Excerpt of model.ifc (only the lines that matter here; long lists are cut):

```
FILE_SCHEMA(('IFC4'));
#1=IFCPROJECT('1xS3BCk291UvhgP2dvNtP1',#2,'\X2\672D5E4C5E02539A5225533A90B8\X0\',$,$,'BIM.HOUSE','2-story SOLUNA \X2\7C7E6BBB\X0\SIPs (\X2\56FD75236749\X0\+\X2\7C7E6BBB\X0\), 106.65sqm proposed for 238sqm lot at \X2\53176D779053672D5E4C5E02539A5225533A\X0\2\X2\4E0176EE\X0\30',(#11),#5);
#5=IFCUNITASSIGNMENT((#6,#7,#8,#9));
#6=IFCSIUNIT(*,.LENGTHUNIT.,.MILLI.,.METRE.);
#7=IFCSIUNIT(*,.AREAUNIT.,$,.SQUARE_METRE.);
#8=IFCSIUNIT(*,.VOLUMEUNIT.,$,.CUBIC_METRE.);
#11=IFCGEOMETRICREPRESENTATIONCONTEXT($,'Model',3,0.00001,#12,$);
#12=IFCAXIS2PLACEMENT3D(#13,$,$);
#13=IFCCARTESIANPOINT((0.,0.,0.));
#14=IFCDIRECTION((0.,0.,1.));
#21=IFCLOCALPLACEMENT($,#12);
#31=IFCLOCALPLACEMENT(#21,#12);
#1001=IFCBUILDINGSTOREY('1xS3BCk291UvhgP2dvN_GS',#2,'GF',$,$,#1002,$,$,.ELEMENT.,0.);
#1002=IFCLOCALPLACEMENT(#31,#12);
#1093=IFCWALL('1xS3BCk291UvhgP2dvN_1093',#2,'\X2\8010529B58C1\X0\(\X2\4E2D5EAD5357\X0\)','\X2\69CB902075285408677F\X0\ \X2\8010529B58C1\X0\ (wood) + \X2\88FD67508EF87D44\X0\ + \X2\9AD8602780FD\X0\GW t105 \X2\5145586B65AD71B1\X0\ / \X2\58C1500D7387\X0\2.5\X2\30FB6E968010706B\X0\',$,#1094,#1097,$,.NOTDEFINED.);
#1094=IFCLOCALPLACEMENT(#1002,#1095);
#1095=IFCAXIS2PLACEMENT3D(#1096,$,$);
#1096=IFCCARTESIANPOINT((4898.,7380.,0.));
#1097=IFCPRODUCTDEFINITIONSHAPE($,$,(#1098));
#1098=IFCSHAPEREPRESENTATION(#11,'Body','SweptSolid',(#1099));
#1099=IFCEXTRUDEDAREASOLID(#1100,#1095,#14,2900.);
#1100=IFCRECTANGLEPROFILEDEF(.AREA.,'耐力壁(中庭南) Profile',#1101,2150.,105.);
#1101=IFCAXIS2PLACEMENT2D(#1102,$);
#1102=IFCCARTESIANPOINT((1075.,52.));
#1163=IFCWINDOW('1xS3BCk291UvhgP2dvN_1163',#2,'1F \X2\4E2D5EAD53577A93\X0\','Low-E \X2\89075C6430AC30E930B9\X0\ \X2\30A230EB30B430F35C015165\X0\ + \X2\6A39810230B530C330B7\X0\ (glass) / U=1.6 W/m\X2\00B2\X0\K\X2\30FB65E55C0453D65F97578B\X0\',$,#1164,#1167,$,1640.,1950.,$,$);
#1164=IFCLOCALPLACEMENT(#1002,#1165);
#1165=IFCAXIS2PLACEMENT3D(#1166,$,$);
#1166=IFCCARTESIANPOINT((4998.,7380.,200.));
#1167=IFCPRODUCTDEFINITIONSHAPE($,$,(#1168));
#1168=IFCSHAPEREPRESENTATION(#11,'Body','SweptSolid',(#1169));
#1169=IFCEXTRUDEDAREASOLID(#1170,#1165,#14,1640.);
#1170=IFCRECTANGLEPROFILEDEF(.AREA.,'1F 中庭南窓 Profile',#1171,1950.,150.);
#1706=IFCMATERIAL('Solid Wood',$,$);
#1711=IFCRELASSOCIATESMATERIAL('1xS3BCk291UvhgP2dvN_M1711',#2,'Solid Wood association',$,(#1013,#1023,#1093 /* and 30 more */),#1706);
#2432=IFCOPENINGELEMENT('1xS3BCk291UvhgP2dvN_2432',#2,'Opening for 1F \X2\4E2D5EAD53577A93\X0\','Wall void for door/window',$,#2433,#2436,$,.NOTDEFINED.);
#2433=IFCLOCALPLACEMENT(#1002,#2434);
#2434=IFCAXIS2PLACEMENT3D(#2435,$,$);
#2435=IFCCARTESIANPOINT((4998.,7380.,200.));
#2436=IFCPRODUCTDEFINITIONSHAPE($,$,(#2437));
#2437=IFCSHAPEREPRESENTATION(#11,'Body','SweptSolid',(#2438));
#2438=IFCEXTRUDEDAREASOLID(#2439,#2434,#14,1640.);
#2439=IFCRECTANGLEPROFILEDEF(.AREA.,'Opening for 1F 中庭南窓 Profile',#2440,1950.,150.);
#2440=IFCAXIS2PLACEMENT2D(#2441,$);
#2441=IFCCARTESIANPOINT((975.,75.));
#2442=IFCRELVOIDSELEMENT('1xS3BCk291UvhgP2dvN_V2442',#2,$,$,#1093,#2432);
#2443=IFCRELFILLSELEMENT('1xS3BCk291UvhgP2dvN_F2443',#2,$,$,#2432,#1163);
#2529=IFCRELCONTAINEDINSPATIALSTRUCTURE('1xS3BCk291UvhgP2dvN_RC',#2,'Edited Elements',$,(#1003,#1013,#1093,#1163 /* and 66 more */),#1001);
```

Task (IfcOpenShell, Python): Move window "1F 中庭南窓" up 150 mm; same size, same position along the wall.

```python
import numpy as np
import ifcopenshell
import ifcopenshell.api.geometry
import ifcopenshell.util.placement
import ifcopenshell.util.unit

model = ifcopenshell.open("model.ifc")
unit_scale = ifcopenshell.util.unit.calculate_unit_scale(model)

window = model.by_guid("1xS3BCk291UvhgP2dvN_1163")
opening = window.FillsVoids[0].RelatingOpeningElement
dz = 150.0

shift = np.array([0.0, 0.0, dz])
# The window is not placed relative to its opening, so move both.
for product in (opening, window):
    matrix = ifcopenshell.util.placement.get_local_placement(product.ObjectPlacement)
    matrix[:3, 3] += shift
    ifcopenshell.api.geometry.edit_object_placement(model, product=product, matrix=matrix, is_si=False)

print(f"moved by {dz * unit_scale:+.3f} m")

model.write("model_rev.ifc")
```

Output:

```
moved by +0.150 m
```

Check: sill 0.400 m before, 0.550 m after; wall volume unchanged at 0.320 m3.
